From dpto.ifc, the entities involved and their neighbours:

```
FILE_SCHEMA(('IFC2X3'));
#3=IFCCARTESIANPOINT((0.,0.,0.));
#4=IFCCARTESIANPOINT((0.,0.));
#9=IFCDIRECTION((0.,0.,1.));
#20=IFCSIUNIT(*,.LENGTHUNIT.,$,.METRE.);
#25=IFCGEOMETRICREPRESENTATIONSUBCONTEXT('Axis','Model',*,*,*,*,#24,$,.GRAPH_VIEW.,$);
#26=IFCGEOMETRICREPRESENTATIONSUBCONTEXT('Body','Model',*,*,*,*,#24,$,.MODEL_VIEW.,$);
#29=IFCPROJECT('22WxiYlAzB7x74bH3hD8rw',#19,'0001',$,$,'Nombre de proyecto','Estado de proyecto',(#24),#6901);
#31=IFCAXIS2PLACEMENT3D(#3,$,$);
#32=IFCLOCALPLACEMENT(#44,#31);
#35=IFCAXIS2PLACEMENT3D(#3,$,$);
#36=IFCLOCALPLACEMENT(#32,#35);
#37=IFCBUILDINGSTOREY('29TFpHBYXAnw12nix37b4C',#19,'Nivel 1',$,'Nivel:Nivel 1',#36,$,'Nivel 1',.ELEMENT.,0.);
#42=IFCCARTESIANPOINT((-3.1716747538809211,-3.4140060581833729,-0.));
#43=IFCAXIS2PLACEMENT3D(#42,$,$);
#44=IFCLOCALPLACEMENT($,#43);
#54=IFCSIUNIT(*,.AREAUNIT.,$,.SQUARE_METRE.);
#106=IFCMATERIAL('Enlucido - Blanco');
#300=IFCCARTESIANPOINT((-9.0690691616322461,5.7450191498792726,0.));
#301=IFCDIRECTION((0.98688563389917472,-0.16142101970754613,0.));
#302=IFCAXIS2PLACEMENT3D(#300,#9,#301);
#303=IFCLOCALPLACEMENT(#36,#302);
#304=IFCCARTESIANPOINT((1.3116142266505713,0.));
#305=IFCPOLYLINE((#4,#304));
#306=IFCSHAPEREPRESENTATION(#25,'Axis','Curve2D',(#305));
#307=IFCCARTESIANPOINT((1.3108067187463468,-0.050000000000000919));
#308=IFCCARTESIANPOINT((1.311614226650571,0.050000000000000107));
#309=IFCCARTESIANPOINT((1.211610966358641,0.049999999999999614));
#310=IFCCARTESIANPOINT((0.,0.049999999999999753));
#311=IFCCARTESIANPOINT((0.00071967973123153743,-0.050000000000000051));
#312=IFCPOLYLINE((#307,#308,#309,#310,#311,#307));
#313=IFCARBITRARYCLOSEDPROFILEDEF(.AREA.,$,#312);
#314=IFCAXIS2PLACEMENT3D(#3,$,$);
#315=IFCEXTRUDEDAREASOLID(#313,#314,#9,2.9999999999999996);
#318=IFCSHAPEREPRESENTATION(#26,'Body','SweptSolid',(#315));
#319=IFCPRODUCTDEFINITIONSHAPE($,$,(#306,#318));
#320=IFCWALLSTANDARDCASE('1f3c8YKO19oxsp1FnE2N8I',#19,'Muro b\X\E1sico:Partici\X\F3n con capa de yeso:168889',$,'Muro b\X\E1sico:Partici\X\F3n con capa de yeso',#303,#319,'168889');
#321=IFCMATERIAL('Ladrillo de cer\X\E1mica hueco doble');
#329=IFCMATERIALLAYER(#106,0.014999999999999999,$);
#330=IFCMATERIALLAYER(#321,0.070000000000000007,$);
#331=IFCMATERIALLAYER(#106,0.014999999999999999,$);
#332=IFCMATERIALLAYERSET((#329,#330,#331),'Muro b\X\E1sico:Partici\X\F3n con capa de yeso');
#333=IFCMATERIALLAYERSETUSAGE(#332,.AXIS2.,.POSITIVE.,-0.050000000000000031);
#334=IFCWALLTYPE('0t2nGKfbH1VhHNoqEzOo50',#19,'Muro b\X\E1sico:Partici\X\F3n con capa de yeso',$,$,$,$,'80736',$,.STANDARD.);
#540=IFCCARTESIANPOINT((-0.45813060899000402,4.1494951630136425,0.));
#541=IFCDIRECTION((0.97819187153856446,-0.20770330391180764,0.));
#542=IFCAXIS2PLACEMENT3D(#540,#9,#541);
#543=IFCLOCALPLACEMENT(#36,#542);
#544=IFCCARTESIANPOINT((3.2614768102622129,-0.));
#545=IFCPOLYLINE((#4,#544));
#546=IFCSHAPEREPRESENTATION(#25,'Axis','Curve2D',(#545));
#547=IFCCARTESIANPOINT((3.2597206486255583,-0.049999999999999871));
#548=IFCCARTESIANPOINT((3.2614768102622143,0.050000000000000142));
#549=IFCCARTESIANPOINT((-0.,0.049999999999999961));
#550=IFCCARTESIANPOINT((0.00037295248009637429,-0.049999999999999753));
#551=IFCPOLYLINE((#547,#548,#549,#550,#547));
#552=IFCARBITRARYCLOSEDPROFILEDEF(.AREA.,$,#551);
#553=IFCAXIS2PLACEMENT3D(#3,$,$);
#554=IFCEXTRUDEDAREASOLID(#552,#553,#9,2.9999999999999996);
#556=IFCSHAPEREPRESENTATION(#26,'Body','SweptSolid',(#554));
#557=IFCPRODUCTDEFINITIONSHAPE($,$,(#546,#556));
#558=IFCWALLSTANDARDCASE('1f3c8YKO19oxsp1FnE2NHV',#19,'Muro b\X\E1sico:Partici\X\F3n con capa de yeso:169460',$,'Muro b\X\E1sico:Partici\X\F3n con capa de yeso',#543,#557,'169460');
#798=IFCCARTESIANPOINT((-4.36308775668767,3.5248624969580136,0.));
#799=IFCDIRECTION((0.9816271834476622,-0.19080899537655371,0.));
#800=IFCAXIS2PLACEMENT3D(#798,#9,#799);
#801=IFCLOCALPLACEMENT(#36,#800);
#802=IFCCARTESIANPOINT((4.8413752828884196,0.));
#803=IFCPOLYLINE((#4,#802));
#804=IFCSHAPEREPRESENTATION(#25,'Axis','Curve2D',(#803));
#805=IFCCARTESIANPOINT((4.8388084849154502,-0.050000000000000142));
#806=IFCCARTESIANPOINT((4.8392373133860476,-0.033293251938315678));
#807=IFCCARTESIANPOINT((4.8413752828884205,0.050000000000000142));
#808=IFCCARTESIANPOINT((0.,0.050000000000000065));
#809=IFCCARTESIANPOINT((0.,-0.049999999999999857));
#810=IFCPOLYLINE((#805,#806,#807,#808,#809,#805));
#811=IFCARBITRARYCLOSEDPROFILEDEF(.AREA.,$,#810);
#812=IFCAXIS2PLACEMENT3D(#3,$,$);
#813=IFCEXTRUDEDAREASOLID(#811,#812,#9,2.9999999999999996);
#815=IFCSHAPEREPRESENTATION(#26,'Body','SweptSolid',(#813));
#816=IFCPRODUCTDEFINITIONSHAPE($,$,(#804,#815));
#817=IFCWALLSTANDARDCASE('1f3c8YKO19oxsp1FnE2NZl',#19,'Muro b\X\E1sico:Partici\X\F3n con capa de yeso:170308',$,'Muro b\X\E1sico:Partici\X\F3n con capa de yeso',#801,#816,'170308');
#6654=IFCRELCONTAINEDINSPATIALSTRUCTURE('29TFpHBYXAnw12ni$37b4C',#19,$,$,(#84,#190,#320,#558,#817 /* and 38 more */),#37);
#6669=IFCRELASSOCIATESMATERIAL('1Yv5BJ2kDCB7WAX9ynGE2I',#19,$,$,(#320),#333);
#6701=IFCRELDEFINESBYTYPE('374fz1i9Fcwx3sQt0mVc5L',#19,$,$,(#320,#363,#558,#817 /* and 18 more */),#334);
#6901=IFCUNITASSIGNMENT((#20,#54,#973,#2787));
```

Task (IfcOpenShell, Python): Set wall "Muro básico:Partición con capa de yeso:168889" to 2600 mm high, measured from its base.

```python
import ifcopenshell
import ifcopenshell.geom
import ifcopenshell.util.representation
import ifcopenshell.util.shape

model = ifcopenshell.open("dpto.ifc")
settings = ifcopenshell.geom.settings()


def volume(element):
    """Net volume in cubic metres, openings subtracted."""
    shape = ifcopenshell.geom.create_shape(settings, element)
    return ifcopenshell.util.shape.get_volume(shape.geometry)


wall = model.by_guid("1f3c8YKO19oxsp1FnE2N8I")
before = volume(wall)

body = ifcopenshell.util.representation.get_representation(wall, "Model", "Body")
solid = body.Items[0]
old_height = solid.Depth
solid.Depth = 2.6
after = volume(wall)

print(f"height {old_height:g} -> {solid.Depth:g}, volume {before:.3f} -> {after:.3f} m3")

model.write("dpto_updated.ifc")
```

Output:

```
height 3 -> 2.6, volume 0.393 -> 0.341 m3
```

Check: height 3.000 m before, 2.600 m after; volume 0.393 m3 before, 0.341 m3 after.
